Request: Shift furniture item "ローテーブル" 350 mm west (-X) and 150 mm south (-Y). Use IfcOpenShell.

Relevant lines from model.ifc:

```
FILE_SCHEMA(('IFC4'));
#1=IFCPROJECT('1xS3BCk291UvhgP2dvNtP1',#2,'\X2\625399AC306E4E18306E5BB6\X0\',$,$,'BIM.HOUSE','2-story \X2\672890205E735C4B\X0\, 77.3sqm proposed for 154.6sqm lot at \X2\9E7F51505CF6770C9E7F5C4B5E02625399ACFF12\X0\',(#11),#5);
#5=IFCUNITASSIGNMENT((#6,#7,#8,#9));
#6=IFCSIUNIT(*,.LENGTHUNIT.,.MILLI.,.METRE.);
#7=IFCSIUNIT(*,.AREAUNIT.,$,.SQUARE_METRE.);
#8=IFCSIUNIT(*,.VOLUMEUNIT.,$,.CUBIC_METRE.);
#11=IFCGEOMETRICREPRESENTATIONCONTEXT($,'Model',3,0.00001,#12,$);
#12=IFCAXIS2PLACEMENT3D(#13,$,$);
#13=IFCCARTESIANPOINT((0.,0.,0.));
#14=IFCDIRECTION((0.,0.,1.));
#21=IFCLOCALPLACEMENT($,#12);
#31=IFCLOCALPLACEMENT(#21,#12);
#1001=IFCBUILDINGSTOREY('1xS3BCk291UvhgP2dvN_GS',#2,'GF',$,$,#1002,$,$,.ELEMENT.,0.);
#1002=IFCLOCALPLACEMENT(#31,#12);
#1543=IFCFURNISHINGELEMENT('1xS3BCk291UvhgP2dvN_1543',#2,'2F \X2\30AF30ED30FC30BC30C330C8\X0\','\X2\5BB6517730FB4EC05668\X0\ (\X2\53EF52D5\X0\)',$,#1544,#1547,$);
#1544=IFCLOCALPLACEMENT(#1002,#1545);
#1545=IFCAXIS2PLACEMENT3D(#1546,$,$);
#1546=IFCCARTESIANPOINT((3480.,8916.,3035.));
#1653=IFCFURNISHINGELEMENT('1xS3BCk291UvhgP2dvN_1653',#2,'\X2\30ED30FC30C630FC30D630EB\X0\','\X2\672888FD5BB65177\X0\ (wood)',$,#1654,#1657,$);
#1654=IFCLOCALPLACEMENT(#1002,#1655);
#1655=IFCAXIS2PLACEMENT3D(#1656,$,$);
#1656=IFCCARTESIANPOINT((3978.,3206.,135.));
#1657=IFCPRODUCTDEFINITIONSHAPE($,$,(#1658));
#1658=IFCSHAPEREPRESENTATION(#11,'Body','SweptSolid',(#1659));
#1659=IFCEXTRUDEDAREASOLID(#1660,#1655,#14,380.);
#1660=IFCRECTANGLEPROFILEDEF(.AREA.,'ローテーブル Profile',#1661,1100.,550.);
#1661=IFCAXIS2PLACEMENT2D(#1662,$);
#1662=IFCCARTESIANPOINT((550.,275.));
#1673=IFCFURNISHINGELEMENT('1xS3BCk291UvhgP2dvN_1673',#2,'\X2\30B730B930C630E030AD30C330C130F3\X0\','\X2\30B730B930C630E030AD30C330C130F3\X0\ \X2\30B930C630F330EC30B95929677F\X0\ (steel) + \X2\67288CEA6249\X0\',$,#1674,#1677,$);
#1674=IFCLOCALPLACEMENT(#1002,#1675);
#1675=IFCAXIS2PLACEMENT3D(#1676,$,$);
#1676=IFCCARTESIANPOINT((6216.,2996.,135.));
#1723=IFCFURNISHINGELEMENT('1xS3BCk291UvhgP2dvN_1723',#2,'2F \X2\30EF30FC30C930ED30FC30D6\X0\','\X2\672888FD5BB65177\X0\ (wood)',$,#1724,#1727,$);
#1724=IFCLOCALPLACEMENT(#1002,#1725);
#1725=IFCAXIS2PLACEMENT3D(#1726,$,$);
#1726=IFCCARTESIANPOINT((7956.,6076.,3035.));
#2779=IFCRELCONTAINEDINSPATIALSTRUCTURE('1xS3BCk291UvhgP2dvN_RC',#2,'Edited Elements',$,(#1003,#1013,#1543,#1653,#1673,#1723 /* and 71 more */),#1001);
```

```python
import ifcopenshell
import ifcopenshell.api.geometry
import ifcopenshell.util.placement
import ifcopenshell.util.unit

model = ifcopenshell.open("model.ifc")
unit_scale = ifcopenshell.util.unit.calculate_unit_scale(model)

item = model.by_guid("1xS3BCk291UvhgP2dvN_1653")
matrix = ifcopenshell.util.placement.get_local_placement(item.ObjectPlacement)
matrix[0, 3] -= 0.35 / unit_scale
matrix[1, 3] -= 0.15 / unit_scale
ifcopenshell.api.geometry.edit_object_placement(model, product=item, matrix=matrix, is_si=False)

print(ifcopenshell.util.placement.get_local_placement(item.ObjectPlacement).round(3) + 0.0)

model.write("model_edited.ifc")
```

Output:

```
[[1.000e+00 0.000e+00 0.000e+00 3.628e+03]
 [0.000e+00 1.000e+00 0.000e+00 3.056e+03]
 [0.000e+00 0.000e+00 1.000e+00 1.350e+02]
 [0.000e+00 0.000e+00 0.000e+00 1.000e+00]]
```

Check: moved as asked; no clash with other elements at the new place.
